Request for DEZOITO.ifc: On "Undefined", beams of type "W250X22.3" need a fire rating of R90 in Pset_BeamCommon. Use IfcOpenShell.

First a look at what the model holds.

```python
import ifcopenshell
import ifcopenshell.util.element

model = ifcopenshell.open("DEZOITO.ifc")
print(model.schema)
storey = next(s for s in model.by_type("IfcBuildingStorey") if s.Name == "Undefined")
beams = [e for e in ifcopenshell.util.element.get_decomposition(storey) if e.is_a("IfcBeam")]
seen = {}
for e in beams:
    element_type = ifcopenshell.util.element.get_type(e)
    key = (element_type.Name if element_type != e and element_type else None, ifcopenshell.util.element.get_pset(e, "Pset_BeamCommon", "FireRating"))
    seen[key] = seen.get(key, 0) + 1
for (name, value), count in sorted(seen.items(), key=str):
    print(count, "x", name, "|", value)
```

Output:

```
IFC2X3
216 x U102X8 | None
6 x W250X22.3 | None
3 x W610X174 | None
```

```python
import ifcopenshell
import ifcopenshell.api.pset
import ifcopenshell.util.element

model = ifcopenshell.open("DEZOITO.ifc")

storey = next(s for s in model.by_type("IfcBuildingStorey") if s.Name == "Undefined")
beams = [e for e in ifcopenshell.util.element.get_decomposition(storey) if e.is_a("IfcBeam")]

count = 0
for e in beams:
    element_type = ifcopenshell.util.element.get_type(e)
    if element_type in (None, e) or element_type.Name != "W250X22.3":
        continue
    found = ifcopenshell.util.element.get_pset(e, "Pset_BeamCommon", should_inherit=False)
    if found:
        pset = model.by_id(found["id"])
        if len(ifcopenshell.util.element.get_elements_by_pset(pset)) > 1:
            pset = ifcopenshell.api.pset.unshare_pset(model, products=[e], pset=pset)[0]
    else:
        pset = ifcopenshell.api.pset.add_pset(model, product=e, name="Pset_BeamCommon")
    ifcopenshell.api.pset.edit_pset(model, pset=pset, properties={"FireRating": "R90"})
    count += 1

print(count, "beams updated")

model.write("DEZOITO_updated.ifc")
```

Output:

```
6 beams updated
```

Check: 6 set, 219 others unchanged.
